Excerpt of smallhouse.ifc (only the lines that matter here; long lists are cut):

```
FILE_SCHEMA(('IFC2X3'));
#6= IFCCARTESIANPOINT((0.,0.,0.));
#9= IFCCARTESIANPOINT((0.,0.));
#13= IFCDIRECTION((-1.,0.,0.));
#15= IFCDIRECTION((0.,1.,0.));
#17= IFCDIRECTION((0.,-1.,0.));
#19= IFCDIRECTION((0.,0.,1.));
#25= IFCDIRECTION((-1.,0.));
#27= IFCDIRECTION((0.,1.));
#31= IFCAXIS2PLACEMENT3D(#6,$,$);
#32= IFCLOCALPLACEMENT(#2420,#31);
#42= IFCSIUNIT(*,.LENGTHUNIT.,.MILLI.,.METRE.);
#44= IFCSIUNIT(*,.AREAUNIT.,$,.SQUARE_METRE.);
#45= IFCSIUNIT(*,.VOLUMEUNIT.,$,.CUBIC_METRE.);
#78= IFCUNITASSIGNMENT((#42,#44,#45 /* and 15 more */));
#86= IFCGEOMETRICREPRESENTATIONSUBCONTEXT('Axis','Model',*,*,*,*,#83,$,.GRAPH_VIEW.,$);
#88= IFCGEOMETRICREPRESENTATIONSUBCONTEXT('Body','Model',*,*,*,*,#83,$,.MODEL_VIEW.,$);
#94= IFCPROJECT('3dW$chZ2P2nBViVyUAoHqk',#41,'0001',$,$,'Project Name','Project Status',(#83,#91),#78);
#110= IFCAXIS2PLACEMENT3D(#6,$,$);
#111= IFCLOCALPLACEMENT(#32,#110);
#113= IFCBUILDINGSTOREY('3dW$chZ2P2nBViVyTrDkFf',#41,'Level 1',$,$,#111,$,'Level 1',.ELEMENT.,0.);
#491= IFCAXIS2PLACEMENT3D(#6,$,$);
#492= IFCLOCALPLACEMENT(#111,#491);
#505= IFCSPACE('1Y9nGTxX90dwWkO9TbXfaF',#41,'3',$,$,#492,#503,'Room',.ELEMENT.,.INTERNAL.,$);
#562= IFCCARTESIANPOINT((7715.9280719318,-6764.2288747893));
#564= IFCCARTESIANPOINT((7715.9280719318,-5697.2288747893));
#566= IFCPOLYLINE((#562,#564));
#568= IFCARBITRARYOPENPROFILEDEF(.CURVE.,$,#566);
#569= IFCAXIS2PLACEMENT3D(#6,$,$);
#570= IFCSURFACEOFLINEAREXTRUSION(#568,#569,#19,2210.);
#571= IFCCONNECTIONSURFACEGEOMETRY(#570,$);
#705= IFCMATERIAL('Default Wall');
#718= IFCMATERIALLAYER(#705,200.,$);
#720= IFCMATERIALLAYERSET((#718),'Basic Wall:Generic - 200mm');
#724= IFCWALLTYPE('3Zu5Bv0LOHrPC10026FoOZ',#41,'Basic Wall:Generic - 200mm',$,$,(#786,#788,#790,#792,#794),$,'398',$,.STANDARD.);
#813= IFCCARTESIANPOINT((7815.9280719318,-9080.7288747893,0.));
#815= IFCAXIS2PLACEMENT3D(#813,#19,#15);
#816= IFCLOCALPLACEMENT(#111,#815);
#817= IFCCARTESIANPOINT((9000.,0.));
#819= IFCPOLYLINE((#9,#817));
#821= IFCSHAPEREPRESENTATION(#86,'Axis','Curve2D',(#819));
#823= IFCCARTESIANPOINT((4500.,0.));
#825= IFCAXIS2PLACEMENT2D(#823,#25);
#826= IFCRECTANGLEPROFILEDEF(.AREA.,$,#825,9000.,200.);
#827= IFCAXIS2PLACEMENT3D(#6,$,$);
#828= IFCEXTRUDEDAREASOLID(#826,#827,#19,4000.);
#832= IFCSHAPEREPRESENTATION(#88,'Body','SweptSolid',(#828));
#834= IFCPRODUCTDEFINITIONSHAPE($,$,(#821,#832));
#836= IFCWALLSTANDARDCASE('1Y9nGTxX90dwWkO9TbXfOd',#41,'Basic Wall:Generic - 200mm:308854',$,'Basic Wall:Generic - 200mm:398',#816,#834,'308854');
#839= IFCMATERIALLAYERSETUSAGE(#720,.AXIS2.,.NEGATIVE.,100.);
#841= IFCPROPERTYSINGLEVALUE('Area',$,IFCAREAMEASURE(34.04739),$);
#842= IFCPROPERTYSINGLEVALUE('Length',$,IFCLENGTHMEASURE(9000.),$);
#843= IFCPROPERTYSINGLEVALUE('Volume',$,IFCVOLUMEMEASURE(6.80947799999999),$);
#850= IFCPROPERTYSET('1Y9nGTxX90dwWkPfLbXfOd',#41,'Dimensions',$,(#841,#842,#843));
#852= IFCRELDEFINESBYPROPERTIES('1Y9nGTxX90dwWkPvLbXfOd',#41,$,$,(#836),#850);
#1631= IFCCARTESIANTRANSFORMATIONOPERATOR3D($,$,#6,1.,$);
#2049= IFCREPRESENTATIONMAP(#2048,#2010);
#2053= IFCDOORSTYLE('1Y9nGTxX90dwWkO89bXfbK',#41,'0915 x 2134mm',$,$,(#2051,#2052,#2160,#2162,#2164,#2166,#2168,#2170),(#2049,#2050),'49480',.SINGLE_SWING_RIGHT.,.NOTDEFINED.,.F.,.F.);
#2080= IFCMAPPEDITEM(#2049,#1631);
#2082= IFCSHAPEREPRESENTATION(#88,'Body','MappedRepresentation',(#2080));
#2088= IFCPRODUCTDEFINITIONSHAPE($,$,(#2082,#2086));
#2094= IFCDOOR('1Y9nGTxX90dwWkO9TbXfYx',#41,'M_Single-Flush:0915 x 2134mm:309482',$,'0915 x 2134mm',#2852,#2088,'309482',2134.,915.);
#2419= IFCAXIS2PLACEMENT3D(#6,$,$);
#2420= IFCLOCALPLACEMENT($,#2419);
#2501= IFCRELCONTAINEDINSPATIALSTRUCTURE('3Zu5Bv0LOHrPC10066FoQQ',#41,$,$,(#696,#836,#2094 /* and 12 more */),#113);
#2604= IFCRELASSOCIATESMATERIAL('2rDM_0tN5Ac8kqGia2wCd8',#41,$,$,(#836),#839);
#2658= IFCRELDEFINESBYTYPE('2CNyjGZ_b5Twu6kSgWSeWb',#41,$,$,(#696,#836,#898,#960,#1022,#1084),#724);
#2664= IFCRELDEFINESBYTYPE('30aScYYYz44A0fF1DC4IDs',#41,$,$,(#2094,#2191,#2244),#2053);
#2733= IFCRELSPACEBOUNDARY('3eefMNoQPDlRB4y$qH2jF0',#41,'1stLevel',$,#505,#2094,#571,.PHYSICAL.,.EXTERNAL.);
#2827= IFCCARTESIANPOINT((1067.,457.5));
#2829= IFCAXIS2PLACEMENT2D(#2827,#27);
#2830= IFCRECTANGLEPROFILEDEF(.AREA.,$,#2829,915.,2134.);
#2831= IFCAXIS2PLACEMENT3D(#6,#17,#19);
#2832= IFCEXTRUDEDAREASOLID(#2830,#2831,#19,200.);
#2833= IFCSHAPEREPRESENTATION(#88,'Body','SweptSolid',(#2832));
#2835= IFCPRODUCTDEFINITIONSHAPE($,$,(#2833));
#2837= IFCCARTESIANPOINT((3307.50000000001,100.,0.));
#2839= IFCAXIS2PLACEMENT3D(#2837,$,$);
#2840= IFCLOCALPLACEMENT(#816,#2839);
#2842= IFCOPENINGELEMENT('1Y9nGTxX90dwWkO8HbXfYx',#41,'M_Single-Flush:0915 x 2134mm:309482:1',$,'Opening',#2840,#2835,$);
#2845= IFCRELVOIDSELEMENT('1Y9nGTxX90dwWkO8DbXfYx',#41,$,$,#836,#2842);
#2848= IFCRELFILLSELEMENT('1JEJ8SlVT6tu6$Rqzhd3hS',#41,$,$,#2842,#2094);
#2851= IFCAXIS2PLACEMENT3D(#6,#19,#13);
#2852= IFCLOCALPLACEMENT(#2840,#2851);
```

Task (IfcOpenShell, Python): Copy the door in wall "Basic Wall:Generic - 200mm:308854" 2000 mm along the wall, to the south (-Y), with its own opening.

```python
import numpy as np
import ifcopenshell
import ifcopenshell.api.feature
import ifcopenshell.api.geometry
import ifcopenshell.api.pset
import ifcopenshell.api.root
import ifcopenshell.geom
import ifcopenshell.util.element
import ifcopenshell.util.placement
import ifcopenshell.util.shape
import ifcopenshell.util.unit

model = ifcopenshell.open("smallhouse.ifc")
area_scale = ifcopenshell.util.unit.calculate_unit_scale(model, "AREAUNIT")
volume_scale = ifcopenshell.util.unit.calculate_unit_scale(model, "VOLUMEUNIT")
settings = ifcopenshell.geom.settings()


def volume(element):
    """Net volume in cubic metres, openings subtracted."""
    shape = ifcopenshell.geom.create_shape(settings, element)
    return ifcopenshell.util.shape.get_volume(shape.geometry)


def reuse_history(source, copy):
    """copy_class also copies each property set's owner history, people and application; keep the originals."""
    for rel in copy.IsDefinedBy:
        if rel.is_a("IfcRelDefinesByProperties") and (history := rel.RelatingPropertyDefinition.OwnerHistory):
            rel.RelatingPropertyDefinition.OwnerHistory = source.OwnerHistory
            ifcopenshell.util.element.remove_deep2(model, history)


door = model.by_id(2094)
opening = door.FillsVoids[0].RelatingOpeningElement
wall = opening.VoidsElements[0].RelatingBuildingElement
before = volume(wall)
shift = ifcopenshell.util.placement.get_local_placement(wall.ObjectPlacement)[:3, 0] * -2000.0

# copy_class copies the void relationship, type, container and properties, but no geometry.
new_opening = ifcopenshell.api.root.copy_class(model, product=opening)
new_opening.Representation = ifcopenshell.util.element.copy_deep(
    model, opening.Representation, exclude=["IfcGeometricRepresentationContext", "IfcRepresentationMap"]
)
new_opening.Name = "M_Single-Flush:0915 x 2134mm"
new_door = ifcopenshell.api.root.copy_class(model, product=door)
new_door.Representation = ifcopenshell.util.element.copy_deep(
    model, door.Representation, exclude=["IfcGeometricRepresentationContext", "IfcRepresentationMap"]
)
new_door.Name = "M_Single-Flush:0915 x 2134mm"
new_door.Tag = None
reuse_history(door, new_door)
fills = ifcopenshell.api.feature.add_filling(model, opening=new_opening, element=new_door)
fills.OwnerHistory = new_door.OwnerHistory  # required in IFC2X3

for old, new in ((opening, new_opening), (door, new_door)):
    matrix = ifcopenshell.util.placement.get_local_placement(old.ObjectPlacement)
    matrix[:3, 3] += shift
    ifcopenshell.api.geometry.edit_object_placement(model, product=new, matrix=matrix, is_si=False)

# The copied space boundaries still share their surfaces with the original.
for rel in new_door.ProvidesBoundaries:
    if rel.ConnectionGeometry:
        rel.ConnectionGeometry = ifcopenshell.util.element.copy_deep(model, rel.ConnectionGeometry)

# Space boundary surfaces are stored in each space's coordinates; move them too.
for rel in new_door.ProvidesBoundaries:
    if not rel.ConnectionGeometry:
        continue
    surface = rel.ConnectionGeometry.SurfaceOnRelatingElement
    space_matrix = ifcopenshell.util.placement.get_local_placement(rel.RelatingSpace.ObjectPlacement)
    point = np.array(surface.Position.Location.Coordinates) + space_matrix[:3, :3].T @ shift
    surface.Position = model.createIfcAxis2Placement3D(
        model.createIfcCartesianPoint(point.tolist()), surface.Position.Axis, surface.Position.RefDirection
    )

after = volume(wall)
thickness = 0.2  # wall thickness in metres

# Update the wall's stored quantities.
pset = model.by_id(ifcopenshell.util.element.get_pset(wall, "Dimensions", should_inherit=False)["id"])
ifcopenshell.api.pset.edit_pset(model, pset=pset, properties={
    "Area": model.create_entity("IfcAreaMeasure", after / thickness / area_scale),
    "Volume": model.create_entity("IfcVolumeMeasure", after / volume_scale),
})

print(f"wall volume {before:.3f} -> {after:.3f} m3")

model.write("smallhouse_rev.ifc")
```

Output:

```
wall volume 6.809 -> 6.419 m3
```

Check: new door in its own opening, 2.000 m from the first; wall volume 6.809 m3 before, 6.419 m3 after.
